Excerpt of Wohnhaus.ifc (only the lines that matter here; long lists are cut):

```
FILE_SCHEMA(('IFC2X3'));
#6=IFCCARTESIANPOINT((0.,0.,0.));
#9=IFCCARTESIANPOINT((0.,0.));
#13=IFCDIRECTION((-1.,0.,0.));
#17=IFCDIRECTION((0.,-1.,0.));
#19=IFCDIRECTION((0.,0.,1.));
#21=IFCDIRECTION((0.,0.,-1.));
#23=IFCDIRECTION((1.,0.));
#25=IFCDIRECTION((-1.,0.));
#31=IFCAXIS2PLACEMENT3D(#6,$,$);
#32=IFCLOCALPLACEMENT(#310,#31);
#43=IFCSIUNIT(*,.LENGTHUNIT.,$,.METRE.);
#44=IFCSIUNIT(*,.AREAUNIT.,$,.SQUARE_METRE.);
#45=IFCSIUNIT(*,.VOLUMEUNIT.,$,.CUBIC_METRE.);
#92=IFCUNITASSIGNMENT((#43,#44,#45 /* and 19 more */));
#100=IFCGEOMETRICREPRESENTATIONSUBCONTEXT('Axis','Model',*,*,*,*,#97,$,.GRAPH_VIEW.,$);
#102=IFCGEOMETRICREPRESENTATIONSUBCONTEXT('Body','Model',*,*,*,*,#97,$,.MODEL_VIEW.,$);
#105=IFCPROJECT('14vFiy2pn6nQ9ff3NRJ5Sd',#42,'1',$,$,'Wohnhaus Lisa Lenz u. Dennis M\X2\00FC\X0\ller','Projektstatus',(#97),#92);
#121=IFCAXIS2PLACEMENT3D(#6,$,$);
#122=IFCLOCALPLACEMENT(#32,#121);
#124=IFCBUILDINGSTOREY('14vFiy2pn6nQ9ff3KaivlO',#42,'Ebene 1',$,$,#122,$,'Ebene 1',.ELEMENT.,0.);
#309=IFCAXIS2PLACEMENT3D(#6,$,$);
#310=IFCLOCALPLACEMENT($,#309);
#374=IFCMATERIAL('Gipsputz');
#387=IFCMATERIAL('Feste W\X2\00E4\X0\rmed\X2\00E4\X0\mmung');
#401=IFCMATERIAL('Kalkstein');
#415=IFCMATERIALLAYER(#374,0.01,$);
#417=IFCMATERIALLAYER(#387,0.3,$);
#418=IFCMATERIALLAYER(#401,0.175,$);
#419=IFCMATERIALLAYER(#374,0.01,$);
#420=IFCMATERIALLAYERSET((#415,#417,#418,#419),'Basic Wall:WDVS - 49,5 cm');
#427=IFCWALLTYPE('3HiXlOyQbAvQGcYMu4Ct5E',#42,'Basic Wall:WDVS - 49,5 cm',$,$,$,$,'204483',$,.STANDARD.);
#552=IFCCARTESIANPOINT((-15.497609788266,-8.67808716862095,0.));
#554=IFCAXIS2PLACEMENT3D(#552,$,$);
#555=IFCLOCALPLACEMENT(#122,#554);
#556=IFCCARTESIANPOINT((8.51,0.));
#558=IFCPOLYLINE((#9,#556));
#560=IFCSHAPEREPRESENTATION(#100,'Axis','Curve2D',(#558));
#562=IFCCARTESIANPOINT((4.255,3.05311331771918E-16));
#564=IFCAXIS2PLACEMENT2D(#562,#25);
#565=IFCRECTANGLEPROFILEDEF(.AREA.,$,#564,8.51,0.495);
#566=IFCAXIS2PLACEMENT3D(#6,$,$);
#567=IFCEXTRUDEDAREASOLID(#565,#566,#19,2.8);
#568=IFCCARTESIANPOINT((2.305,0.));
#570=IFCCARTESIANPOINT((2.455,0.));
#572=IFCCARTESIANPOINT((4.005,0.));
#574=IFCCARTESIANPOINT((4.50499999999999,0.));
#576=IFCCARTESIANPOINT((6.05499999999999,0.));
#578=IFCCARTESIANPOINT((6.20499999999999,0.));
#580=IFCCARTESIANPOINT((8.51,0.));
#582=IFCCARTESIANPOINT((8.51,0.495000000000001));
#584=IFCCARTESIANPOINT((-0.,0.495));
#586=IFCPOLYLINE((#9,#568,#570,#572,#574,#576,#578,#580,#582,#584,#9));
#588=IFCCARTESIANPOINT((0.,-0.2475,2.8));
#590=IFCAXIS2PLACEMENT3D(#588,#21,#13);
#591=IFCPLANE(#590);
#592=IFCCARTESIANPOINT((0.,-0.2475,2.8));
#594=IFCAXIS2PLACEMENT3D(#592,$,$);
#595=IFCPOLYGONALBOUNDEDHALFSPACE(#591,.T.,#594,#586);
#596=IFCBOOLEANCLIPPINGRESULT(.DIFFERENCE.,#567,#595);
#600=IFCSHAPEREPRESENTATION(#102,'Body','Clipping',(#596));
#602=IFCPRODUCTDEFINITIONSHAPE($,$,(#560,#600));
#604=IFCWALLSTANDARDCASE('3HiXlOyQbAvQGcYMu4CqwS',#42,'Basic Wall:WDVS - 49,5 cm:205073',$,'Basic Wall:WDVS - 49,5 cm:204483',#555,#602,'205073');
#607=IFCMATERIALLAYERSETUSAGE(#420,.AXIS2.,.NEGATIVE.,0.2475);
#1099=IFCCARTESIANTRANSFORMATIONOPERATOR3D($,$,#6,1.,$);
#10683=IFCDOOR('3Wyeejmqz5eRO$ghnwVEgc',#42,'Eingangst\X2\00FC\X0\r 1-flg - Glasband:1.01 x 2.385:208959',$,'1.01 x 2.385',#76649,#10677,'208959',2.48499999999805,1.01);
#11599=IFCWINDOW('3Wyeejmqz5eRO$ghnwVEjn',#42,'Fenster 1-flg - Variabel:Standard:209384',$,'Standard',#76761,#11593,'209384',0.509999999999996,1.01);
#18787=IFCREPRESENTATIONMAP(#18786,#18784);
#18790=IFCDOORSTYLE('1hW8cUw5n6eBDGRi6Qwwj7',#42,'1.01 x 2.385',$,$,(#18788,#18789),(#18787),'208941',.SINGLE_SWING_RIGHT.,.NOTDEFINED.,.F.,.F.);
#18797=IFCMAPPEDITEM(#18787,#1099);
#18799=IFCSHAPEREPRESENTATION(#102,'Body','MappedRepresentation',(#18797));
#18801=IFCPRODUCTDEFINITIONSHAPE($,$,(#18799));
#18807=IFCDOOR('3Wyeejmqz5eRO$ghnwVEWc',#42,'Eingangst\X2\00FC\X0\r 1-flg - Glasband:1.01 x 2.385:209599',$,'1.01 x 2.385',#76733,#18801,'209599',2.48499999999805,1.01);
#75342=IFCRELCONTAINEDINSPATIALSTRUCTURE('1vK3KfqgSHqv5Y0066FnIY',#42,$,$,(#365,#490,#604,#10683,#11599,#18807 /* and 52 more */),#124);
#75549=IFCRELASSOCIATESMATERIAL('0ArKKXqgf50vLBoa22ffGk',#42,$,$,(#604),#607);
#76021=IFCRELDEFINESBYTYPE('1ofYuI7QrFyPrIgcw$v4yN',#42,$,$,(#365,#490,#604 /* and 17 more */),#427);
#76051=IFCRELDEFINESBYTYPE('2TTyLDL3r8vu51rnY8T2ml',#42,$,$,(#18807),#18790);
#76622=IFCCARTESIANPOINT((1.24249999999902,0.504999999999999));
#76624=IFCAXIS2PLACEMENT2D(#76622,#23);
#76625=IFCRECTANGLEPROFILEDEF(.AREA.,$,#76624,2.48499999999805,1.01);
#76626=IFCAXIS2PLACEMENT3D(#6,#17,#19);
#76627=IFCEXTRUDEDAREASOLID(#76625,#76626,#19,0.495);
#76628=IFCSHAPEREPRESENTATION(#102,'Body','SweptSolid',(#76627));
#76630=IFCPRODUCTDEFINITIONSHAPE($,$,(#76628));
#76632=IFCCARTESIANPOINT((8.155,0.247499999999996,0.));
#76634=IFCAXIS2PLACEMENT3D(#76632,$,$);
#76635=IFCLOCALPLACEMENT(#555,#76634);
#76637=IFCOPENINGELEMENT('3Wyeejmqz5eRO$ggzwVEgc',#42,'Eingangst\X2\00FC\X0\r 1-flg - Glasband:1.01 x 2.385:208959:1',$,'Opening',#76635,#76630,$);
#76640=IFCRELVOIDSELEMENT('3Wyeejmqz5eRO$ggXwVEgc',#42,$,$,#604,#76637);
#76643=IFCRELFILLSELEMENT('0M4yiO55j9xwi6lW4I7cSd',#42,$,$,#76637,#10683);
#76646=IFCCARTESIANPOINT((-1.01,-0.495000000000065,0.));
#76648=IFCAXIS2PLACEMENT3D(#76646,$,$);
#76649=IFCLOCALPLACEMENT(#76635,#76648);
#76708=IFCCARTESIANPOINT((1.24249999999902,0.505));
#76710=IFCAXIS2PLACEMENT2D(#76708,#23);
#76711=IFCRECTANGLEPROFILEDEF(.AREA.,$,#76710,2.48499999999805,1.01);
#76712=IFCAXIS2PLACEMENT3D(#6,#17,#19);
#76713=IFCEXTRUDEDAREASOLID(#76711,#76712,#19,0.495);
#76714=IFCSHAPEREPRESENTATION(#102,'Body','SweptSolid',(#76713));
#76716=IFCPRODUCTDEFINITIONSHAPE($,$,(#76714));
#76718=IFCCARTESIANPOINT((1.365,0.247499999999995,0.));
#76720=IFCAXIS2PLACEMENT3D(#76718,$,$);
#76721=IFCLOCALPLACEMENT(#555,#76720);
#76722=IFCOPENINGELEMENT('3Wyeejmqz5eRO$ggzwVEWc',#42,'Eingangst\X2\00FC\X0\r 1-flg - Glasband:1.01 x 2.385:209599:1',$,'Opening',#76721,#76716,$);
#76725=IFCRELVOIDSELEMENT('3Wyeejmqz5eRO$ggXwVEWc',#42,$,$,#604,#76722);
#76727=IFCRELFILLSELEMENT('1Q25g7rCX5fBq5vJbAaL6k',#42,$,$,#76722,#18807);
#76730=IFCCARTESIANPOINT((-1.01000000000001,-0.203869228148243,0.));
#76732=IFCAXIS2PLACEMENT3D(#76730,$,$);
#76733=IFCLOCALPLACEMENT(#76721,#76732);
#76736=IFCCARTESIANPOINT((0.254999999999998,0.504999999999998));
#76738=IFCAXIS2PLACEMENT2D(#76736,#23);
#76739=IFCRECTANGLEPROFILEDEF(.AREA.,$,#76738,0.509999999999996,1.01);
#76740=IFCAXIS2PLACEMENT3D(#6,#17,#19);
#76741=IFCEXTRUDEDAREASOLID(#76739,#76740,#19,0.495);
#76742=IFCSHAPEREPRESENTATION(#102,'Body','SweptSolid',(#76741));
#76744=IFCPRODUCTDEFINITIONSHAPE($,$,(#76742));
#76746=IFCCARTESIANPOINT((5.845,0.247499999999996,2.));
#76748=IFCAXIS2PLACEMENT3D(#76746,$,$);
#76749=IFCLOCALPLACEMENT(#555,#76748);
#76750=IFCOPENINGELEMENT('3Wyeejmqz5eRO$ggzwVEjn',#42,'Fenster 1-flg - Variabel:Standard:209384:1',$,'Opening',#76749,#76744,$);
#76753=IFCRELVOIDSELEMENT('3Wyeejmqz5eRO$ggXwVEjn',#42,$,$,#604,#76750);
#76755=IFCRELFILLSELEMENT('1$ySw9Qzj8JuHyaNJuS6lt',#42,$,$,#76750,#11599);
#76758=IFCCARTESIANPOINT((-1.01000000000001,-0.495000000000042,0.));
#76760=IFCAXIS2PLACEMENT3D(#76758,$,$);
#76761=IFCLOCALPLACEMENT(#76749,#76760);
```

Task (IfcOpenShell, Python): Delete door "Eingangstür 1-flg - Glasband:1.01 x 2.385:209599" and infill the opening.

```python
import ifcopenshell
import ifcopenshell.api.feature
import ifcopenshell.api.root
import ifcopenshell.geom
import ifcopenshell.util.shape

model = ifcopenshell.open("Wohnhaus.ifc")
settings = ifcopenshell.geom.settings()


def volume(element):
    """Net volume in cubic metres, openings subtracted."""
    shape = ifcopenshell.geom.create_shape(settings, element)
    return ifcopenshell.util.shape.get_volume(shape.geometry)


door = model.by_guid("3Wyeejmqz5eRO$ghnwVEWc")
opening = door.FillsVoids[0].RelatingOpeningElement
wall = opening.VoidsElements[0].RelatingBuildingElement
before = volume(wall)

ifcopenshell.api.root.remove_product(model, product=door)
ifcopenshell.api.feature.remove_feature(model, feature=opening)

after = volume(wall)

print(f"wall volume {before:.3f} -> {after:.3f} m3")

model.write("Wohnhaus_v2.ifc")
```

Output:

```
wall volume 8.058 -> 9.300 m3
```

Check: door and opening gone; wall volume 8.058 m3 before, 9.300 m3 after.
